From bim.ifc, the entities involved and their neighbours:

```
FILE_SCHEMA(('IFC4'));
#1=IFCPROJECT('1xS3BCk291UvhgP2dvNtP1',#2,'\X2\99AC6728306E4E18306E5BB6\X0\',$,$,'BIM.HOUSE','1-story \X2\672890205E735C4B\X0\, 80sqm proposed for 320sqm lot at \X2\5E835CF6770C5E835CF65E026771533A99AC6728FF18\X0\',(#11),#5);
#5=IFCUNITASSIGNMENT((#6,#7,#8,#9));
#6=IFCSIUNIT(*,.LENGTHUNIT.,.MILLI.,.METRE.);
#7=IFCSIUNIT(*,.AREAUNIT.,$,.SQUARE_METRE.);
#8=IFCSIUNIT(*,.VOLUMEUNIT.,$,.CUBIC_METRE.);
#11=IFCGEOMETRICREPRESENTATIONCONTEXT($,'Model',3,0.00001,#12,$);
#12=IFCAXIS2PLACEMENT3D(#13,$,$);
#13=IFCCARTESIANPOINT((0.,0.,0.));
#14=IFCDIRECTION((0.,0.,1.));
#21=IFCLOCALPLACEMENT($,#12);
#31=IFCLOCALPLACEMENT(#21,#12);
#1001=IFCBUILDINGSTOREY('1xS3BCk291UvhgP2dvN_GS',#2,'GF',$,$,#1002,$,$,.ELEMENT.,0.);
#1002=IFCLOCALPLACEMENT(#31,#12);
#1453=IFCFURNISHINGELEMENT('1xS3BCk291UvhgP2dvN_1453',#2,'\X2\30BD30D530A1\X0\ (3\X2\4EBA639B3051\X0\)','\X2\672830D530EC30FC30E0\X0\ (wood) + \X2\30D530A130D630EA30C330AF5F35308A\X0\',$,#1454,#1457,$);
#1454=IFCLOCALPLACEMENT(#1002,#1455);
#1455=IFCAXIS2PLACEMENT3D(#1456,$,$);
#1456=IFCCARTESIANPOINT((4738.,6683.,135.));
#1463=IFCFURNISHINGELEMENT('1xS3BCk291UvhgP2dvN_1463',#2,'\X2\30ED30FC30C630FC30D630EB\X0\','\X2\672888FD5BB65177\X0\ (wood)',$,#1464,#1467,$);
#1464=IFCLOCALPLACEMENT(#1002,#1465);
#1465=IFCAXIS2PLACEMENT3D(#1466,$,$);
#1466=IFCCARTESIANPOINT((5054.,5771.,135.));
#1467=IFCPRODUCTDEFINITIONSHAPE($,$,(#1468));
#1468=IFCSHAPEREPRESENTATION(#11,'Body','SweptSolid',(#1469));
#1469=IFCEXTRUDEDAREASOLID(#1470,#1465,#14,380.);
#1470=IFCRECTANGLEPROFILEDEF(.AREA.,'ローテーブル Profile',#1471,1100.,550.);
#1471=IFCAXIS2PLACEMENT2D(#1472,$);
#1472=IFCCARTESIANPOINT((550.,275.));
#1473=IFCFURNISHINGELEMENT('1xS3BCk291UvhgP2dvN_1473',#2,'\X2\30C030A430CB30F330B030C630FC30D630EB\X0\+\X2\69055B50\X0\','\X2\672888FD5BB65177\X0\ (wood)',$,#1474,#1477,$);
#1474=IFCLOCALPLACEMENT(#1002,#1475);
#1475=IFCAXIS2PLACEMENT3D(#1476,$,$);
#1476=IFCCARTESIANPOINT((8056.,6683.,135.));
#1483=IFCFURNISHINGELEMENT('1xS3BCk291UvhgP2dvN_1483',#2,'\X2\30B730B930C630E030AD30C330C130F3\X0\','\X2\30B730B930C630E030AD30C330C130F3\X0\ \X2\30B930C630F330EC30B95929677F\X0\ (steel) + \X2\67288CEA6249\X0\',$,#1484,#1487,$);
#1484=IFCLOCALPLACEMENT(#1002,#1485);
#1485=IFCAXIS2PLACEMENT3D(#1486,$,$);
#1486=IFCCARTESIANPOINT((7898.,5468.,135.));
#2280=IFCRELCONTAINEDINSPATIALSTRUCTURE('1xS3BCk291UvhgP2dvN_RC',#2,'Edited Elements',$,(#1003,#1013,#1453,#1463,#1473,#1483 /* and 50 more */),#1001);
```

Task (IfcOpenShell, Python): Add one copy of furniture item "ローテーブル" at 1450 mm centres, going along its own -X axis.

```python
import ifcopenshell
import ifcopenshell.api.geometry
import ifcopenshell.api.root
import ifcopenshell.util.element
import ifcopenshell.util.placement

model = ifcopenshell.open("bim.ifc")


def reuse_history(source, copy):
    """copy_class also copies each property set's owner history, people and application; keep the originals."""
    for rel in copy.IsDefinedBy:
        if rel.is_a("IfcRelDefinesByProperties") and (history := rel.RelatingPropertyDefinition.OwnerHistory):
            rel.RelatingPropertyDefinition.OwnerHistory = source.OwnerHistory
            ifcopenshell.util.element.remove_deep2(model, history)


source = model.by_id(1463)
base = ifcopenshell.util.placement.get_local_placement(source.ObjectPlacement)
step = -base[:3, 0] * 1450.0

for i in range(1, 2):
    copy = ifcopenshell.api.root.copy_class(model, product=source)
    copy.Representation = ifcopenshell.util.element.copy_deep(
        model, source.Representation, exclude=["IfcGeometricRepresentationContext", "IfcRepresentationMap"]
    )
    reuse_history(source, copy)
    matrix = base.copy()
    matrix[:3, 3] += i * step
    print("added at", matrix[:3, 3].round(3) + 0.0)
    ifcopenshell.api.geometry.edit_object_placement(model, product=copy, matrix=matrix, is_si=False)

model.write("bim_rev.ifc")
```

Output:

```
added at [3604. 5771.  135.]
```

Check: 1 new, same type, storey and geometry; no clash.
